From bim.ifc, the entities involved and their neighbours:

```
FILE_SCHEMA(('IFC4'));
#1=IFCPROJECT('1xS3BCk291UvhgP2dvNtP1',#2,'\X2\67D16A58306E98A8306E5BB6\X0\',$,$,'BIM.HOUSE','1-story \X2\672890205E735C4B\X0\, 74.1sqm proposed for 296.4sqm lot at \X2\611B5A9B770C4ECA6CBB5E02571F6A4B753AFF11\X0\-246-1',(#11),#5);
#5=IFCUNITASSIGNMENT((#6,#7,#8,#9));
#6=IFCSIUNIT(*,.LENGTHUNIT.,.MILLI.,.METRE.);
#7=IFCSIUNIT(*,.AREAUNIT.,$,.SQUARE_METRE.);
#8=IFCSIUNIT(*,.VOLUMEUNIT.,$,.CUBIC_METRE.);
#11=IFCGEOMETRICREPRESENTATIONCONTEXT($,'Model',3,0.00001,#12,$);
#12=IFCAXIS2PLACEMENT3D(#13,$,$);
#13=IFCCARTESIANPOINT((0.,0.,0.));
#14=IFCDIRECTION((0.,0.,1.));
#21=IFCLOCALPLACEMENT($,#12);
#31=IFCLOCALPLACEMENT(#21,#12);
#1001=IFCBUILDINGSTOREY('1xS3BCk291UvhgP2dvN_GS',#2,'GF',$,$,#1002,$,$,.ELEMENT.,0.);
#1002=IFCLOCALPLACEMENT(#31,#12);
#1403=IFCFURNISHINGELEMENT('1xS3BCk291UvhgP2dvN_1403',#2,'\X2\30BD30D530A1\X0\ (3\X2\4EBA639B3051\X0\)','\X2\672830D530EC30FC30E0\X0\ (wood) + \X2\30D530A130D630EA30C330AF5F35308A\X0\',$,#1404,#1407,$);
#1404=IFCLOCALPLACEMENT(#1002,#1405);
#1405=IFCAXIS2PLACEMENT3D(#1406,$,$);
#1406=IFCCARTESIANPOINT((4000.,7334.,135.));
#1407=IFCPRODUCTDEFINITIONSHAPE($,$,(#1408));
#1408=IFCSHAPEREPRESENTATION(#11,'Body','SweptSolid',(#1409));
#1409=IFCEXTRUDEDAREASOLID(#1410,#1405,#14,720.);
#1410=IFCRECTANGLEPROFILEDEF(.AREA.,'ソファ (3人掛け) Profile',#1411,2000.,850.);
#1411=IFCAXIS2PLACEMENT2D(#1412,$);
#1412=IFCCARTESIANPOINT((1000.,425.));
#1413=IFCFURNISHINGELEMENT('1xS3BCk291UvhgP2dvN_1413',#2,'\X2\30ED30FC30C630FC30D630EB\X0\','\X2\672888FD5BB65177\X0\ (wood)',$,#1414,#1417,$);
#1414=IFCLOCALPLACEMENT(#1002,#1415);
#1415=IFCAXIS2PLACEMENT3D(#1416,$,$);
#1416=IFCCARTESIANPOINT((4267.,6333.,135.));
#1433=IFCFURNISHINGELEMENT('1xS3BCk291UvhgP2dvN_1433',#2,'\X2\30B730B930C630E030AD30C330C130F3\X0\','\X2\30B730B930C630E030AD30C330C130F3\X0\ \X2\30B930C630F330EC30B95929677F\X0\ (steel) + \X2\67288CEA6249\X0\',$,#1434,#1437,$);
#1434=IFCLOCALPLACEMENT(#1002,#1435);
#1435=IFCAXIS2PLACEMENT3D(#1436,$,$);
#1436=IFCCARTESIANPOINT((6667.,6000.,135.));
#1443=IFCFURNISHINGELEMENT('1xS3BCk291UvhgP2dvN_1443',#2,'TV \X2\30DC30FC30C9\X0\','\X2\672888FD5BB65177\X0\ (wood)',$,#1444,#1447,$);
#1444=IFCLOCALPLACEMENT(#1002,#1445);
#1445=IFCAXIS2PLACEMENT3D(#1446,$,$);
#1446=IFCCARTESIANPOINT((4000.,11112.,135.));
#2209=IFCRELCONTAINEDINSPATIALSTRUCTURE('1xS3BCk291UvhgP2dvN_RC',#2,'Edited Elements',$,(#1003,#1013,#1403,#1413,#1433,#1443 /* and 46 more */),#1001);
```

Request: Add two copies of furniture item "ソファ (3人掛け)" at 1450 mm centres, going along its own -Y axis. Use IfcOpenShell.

```python
import ifcopenshell
import ifcopenshell.api.geometry
import ifcopenshell.api.root
import ifcopenshell.util.element
import ifcopenshell.util.placement

model = ifcopenshell.open("bim.ifc")


def reuse_history(source, copy):
    """copy_class also copies each property set's owner history, people and application; keep the originals."""
    for rel in copy.IsDefinedBy:
        if rel.is_a("IfcRelDefinesByProperties") and (history := rel.RelatingPropertyDefinition.OwnerHistory):
            rel.RelatingPropertyDefinition.OwnerHistory = source.OwnerHistory
            ifcopenshell.util.element.remove_deep2(model, history)


source = model.by_guid("1xS3BCk291UvhgP2dvN_1403")
base = ifcopenshell.util.placement.get_local_placement(source.ObjectPlacement)
step = -base[:3, 1] * 1450.0

for i in range(1, 3):
    copy = ifcopenshell.api.root.copy_class(model, product=source)
    copy.Representation = ifcopenshell.util.element.copy_deep(
        model, source.Representation, exclude=["IfcGeometricRepresentationContext", "IfcRepresentationMap"]
    )
    reuse_history(source, copy)
    matrix = base.copy()
    matrix[:3, 3] += i * step
    print("added at", matrix[:3, 3].round(3) + 0.0)
    ifcopenshell.api.geometry.edit_object_placement(model, product=copy, matrix=matrix, is_si=False)

model.write("bim_v2.ifc")
```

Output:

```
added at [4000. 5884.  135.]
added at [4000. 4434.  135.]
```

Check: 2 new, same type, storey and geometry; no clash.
